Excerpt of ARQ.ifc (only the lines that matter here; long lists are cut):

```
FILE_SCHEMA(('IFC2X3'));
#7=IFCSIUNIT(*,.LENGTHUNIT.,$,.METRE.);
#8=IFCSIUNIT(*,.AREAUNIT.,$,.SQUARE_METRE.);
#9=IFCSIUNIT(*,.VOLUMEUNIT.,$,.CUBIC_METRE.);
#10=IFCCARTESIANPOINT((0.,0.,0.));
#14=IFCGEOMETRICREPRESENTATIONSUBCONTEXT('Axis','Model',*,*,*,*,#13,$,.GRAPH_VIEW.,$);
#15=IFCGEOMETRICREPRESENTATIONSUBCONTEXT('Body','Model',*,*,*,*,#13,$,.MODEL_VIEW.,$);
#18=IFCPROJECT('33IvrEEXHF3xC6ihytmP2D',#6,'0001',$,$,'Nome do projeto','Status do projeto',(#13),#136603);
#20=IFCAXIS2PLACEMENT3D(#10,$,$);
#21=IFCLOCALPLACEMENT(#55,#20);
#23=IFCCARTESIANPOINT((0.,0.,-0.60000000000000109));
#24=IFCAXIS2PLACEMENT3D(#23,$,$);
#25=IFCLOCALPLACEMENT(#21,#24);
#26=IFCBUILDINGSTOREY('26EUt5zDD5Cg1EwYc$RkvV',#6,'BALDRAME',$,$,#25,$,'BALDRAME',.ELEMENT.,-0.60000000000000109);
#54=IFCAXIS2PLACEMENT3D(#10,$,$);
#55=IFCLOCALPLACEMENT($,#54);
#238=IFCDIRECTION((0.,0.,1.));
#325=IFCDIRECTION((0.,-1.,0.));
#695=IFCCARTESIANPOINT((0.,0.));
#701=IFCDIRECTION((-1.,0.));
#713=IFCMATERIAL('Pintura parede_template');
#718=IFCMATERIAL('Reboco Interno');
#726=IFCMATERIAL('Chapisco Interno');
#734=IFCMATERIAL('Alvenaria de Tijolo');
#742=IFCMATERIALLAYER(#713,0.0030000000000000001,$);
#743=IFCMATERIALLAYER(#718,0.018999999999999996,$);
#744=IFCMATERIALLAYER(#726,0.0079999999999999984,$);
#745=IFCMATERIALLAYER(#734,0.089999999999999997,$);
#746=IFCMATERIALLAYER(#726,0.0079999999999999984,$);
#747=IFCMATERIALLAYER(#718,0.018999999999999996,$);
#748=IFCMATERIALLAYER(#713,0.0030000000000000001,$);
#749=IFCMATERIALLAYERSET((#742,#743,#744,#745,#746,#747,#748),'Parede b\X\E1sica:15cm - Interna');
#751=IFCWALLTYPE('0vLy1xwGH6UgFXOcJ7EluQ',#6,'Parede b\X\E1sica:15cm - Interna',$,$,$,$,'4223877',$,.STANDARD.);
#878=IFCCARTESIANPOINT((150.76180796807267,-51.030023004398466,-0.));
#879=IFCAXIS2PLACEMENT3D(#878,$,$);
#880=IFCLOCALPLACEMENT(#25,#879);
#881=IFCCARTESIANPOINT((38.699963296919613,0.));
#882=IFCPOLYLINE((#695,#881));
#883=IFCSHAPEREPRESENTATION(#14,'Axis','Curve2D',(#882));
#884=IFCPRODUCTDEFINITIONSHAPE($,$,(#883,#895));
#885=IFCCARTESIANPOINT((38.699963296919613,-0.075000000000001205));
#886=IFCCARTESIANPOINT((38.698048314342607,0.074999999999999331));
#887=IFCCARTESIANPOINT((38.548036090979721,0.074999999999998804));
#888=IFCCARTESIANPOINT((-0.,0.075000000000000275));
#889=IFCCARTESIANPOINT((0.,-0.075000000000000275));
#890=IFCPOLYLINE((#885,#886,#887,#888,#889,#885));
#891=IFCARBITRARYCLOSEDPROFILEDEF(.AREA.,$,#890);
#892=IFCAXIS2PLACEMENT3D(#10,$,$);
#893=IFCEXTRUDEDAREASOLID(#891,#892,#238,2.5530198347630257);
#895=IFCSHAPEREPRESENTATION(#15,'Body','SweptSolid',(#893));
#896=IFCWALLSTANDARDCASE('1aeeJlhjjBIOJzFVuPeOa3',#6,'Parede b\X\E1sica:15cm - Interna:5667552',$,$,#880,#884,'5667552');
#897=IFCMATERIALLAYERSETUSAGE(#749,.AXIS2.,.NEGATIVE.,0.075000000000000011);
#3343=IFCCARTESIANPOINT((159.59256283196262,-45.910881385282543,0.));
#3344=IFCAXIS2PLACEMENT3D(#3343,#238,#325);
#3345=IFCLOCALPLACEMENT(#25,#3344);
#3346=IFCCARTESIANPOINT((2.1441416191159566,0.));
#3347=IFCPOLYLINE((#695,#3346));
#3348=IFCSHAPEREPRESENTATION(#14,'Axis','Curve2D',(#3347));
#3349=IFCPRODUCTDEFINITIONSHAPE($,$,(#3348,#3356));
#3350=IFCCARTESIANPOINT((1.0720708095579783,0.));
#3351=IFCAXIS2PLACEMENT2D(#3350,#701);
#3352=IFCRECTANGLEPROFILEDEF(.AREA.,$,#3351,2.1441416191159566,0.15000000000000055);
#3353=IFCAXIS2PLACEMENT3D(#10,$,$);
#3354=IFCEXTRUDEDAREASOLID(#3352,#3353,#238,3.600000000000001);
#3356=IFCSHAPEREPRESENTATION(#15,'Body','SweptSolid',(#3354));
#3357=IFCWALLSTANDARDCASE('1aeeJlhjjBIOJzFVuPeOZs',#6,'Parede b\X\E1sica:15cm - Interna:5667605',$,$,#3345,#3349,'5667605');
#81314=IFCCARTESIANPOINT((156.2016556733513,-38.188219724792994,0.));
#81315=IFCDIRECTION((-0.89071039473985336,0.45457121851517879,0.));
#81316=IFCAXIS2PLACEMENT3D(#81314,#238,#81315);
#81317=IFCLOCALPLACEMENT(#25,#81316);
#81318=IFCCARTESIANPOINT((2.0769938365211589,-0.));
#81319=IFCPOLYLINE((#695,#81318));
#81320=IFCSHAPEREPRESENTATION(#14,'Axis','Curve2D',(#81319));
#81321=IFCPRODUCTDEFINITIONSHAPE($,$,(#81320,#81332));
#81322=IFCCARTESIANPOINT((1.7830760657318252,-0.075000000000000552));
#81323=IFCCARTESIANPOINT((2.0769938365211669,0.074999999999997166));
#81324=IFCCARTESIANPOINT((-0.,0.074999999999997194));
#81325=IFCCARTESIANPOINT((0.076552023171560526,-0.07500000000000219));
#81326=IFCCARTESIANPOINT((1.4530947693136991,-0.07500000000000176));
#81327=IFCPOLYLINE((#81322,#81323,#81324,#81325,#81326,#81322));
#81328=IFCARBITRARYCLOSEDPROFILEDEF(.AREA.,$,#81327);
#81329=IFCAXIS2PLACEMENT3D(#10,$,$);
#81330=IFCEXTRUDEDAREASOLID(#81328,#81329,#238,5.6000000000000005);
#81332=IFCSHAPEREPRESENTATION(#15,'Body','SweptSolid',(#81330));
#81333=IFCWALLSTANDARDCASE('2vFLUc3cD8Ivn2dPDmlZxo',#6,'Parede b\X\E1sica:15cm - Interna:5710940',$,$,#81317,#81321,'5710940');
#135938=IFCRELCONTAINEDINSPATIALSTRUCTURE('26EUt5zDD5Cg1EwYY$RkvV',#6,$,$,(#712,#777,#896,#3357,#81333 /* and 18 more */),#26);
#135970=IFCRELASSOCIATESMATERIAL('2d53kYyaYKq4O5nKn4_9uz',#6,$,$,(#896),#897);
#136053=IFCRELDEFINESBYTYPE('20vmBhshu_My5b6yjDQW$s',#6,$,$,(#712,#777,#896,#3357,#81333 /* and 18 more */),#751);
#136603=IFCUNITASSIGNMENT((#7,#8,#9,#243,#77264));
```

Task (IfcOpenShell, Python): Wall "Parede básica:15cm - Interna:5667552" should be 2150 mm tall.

```python
import ifcopenshell
import ifcopenshell.geom
import ifcopenshell.util.representation
import ifcopenshell.util.shape
import ifcopenshell.util.unit

model = ifcopenshell.open("ARQ.ifc")
unit_scale = ifcopenshell.util.unit.calculate_unit_scale(model)
settings = ifcopenshell.geom.settings()


def volume(element):
    """Net volume in cubic metres, openings subtracted."""
    shape = ifcopenshell.geom.create_shape(settings, element)
    return ifcopenshell.util.shape.get_volume(shape.geometry)


wall = model.by_guid("1aeeJlhjjBIOJzFVuPeOa3")
before = volume(wall)

body = ifcopenshell.util.representation.get_representation(wall, "Model", "Body")
solid = body.Items[0]
old_height = solid.Depth
solid.Depth = 2.15 / unit_scale
after = volume(wall)

print(f"height {old_height:g} -> {solid.Depth:g}, volume {before:.3f} -> {after:.3f} m3")

model.write("ARQ-out.ifc")
```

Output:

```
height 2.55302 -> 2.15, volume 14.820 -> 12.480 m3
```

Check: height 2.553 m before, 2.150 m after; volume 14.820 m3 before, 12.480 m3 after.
